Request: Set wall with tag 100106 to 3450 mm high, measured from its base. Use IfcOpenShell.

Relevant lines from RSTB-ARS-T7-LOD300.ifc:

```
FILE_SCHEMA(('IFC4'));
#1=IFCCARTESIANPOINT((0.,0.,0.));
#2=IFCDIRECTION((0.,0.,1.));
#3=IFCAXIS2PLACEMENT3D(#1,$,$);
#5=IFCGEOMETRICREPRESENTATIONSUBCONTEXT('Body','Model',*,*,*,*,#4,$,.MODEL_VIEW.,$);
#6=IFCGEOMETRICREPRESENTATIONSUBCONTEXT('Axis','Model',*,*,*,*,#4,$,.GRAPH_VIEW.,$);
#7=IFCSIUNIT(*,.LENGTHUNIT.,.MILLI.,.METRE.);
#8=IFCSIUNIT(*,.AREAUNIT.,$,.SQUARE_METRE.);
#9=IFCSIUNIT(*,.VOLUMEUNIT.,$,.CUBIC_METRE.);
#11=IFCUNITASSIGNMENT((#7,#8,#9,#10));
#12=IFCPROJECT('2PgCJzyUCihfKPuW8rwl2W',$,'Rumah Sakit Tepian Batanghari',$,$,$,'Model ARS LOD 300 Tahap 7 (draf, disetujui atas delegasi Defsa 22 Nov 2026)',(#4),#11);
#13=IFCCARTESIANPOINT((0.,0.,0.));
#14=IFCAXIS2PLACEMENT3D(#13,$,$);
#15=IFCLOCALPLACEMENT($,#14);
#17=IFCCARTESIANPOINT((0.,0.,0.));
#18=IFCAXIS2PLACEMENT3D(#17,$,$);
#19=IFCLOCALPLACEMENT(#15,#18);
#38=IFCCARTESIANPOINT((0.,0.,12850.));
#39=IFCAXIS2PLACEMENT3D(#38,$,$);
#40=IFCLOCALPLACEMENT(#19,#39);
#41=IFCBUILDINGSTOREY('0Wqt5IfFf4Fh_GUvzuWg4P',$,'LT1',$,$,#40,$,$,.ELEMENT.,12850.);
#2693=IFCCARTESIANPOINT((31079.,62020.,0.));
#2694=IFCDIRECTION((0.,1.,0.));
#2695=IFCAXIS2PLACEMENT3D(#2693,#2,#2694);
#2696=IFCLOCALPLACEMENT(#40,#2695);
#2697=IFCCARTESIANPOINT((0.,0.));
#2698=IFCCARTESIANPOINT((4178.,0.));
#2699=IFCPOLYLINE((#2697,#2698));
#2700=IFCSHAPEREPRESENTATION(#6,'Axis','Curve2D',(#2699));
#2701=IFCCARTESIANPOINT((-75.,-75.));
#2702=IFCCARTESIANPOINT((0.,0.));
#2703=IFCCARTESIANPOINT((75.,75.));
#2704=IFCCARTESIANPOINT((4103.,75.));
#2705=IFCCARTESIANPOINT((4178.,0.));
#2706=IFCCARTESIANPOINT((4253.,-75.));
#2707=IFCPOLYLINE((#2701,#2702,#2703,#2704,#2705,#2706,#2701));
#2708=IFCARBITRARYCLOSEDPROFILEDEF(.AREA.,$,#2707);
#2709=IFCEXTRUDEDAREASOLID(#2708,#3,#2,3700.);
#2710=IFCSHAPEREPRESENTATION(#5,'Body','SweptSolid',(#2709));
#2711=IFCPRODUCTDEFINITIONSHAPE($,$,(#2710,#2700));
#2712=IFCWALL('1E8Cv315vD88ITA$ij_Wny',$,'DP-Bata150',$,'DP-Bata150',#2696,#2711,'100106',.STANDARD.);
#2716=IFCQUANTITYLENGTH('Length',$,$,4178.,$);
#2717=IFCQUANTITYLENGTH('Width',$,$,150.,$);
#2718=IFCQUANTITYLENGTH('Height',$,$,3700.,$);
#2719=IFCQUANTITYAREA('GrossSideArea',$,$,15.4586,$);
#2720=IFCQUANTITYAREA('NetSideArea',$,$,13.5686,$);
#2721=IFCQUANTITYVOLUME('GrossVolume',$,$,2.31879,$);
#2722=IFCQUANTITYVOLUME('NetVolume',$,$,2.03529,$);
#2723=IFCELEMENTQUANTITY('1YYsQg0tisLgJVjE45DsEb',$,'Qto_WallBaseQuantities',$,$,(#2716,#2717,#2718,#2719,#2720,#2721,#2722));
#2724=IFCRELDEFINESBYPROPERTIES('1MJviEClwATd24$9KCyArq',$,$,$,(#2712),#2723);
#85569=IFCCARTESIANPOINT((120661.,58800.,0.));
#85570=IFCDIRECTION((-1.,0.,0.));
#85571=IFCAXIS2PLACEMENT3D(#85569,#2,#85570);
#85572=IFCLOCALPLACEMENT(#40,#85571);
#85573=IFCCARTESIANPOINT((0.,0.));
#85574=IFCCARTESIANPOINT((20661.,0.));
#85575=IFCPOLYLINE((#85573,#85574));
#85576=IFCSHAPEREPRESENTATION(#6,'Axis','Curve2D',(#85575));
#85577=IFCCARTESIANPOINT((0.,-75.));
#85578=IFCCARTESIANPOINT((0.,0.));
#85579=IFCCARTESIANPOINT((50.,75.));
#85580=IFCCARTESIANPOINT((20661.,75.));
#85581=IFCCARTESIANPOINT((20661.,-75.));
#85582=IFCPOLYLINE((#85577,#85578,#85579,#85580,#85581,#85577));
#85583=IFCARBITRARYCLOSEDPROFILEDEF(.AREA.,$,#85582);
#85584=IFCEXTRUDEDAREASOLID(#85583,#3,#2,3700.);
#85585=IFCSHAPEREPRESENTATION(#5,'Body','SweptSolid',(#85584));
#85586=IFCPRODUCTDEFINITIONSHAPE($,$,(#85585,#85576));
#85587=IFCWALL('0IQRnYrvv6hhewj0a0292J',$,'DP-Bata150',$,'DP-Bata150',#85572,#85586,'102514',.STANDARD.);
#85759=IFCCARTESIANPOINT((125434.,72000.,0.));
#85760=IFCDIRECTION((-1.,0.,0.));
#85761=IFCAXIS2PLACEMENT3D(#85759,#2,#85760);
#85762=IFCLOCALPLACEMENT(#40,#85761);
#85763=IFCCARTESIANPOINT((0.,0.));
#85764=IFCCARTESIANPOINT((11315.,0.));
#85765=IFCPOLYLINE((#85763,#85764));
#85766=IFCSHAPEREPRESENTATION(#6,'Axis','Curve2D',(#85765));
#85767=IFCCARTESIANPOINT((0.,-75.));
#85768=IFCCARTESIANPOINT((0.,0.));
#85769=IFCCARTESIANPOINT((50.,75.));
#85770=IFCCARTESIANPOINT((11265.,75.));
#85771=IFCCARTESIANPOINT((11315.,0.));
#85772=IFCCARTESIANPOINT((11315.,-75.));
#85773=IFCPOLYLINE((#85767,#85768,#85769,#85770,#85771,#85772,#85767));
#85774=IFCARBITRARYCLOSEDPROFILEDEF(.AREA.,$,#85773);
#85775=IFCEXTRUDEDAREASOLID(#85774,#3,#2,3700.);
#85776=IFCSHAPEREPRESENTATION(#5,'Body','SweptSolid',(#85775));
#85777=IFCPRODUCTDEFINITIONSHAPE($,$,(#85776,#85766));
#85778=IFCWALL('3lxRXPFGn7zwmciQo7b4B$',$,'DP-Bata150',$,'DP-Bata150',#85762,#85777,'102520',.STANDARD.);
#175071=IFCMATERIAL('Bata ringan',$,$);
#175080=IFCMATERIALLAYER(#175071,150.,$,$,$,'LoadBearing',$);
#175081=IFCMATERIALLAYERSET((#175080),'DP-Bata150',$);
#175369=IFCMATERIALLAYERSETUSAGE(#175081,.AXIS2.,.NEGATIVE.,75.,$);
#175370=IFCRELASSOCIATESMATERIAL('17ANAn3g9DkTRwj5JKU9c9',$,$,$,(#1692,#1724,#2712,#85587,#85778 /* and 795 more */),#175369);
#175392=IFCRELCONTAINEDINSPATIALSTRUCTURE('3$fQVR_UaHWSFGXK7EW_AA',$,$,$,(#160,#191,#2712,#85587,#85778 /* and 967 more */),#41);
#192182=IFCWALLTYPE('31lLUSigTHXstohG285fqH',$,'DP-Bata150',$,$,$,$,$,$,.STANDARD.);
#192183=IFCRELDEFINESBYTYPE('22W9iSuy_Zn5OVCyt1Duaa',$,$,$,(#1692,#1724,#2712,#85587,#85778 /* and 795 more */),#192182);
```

```python
import ifcopenshell
import ifcopenshell.api.pset
import ifcopenshell.geom
import ifcopenshell.util.element
import ifcopenshell.util.representation
import ifcopenshell.util.shape
import ifcopenshell.util.unit

model = ifcopenshell.open("RSTB-ARS-T7-LOD300.ifc")
unit_scale = ifcopenshell.util.unit.calculate_unit_scale(model)
area_scale = ifcopenshell.util.unit.calculate_unit_scale(model, "AREAUNIT")
volume_scale = ifcopenshell.util.unit.calculate_unit_scale(model, "VOLUMEUNIT")
settings = ifcopenshell.geom.settings()


def volume(element):
    """Net volume in cubic metres, openings subtracted."""
    shape = ifcopenshell.geom.create_shape(settings, element)
    return ifcopenshell.util.shape.get_volume(shape.geometry)


wall = model.by_guid("1E8Cv315vD88ITA$ij_Wny")
before = volume(wall)

body = ifcopenshell.util.representation.get_representation(wall, "Model", "Body")
solid = body.Items[0]
old_height = solid.Depth
solid.Depth = 3.45 / unit_scale
after = volume(wall)
thickness = 0.15  # wall thickness in metres

# Update the stored height, areas and volumes.
qto = model.by_id(ifcopenshell.util.element.get_pset(wall, "Qto_WallBaseQuantities", should_inherit=False)["id"])
ifcopenshell.api.pset.edit_qto(model, qto=qto, properties={
    "Height": solid.Depth,
    "GrossSideArea": ifcopenshell.util.element.get_pset(wall, "Qto_WallBaseQuantities", "GrossSideArea") * solid.Depth / old_height,
    "NetSideArea": after / thickness / area_scale,
    "GrossVolume": ifcopenshell.util.element.get_pset(wall, "Qto_WallBaseQuantities", "GrossVolume") * solid.Depth / old_height,
    "NetVolume": after / volume_scale,
})

print(f"height {old_height:g} -> {solid.Depth:g}, volume {before:.3f} -> {after:.3f} m3")

model.write("RSTB-ARS-T7-LOD300_rev.ifc")
```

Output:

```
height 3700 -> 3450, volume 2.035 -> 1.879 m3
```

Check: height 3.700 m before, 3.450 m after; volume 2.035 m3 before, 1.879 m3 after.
